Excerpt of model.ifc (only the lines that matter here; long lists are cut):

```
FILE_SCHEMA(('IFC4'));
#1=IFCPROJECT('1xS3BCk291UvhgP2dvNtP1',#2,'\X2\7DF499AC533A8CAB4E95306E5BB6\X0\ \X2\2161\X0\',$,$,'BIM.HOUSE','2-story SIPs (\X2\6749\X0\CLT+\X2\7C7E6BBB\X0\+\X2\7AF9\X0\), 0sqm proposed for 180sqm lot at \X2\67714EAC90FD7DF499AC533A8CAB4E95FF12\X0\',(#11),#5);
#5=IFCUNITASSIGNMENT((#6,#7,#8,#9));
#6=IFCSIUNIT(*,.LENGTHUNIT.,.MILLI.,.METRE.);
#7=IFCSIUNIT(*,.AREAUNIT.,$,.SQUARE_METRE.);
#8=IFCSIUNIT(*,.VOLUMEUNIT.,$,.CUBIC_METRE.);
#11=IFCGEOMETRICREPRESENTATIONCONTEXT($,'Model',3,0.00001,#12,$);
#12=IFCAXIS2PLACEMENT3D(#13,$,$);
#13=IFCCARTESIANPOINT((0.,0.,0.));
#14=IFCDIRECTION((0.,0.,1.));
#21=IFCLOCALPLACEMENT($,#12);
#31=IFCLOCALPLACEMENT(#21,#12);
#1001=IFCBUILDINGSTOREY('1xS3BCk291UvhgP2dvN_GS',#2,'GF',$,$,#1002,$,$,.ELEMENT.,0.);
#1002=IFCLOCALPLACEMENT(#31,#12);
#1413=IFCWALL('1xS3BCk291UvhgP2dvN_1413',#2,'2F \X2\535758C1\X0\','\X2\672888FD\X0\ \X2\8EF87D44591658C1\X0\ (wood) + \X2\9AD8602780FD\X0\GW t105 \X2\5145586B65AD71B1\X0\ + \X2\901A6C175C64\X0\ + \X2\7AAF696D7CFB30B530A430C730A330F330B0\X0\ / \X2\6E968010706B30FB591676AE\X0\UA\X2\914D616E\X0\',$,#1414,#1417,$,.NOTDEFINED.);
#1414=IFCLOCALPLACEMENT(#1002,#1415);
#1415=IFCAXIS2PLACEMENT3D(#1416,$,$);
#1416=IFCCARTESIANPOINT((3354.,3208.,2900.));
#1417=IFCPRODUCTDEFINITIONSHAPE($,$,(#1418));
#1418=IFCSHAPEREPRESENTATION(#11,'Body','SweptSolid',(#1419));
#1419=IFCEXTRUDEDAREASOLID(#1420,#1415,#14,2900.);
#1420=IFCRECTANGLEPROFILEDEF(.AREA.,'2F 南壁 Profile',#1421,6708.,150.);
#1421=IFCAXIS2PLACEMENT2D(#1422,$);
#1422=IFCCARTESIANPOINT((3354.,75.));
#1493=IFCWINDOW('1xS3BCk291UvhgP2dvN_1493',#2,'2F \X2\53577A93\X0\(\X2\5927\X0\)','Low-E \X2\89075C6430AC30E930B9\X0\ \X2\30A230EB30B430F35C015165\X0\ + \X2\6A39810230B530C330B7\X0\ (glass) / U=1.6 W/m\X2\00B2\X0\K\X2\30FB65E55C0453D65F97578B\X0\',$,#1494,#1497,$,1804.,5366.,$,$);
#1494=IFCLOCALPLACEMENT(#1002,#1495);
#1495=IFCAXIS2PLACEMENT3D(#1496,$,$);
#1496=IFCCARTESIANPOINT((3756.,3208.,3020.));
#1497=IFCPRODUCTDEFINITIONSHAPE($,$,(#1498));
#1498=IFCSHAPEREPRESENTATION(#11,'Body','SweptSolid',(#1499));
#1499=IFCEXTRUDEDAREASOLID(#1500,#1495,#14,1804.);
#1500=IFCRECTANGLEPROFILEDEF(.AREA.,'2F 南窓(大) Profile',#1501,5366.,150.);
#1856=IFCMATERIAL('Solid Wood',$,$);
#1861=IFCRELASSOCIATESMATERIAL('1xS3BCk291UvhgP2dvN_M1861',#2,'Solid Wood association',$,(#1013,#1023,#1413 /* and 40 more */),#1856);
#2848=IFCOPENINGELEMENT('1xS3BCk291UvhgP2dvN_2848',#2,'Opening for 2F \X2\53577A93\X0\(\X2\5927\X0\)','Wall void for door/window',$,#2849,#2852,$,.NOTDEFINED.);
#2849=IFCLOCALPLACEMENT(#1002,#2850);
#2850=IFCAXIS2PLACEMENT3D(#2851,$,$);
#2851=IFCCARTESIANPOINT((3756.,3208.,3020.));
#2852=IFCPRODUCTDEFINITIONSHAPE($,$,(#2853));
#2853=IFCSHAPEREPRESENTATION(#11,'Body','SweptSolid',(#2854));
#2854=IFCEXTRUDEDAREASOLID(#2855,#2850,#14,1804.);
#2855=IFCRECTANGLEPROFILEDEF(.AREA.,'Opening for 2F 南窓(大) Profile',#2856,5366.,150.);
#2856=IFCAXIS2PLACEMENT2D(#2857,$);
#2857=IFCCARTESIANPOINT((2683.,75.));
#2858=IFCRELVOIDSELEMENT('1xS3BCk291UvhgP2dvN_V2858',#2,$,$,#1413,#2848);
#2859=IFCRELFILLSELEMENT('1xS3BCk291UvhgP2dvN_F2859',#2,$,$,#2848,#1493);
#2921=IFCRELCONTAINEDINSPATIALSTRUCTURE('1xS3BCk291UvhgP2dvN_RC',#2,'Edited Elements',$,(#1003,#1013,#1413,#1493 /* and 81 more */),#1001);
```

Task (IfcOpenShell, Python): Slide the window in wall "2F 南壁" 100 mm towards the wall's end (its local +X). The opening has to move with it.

```python
import ifcopenshell
import ifcopenshell.api.geometry
import ifcopenshell.util.placement
import ifcopenshell.util.unit

model = ifcopenshell.open("model.ifc")
unit_scale = ifcopenshell.util.unit.calculate_unit_scale(model)

window = model.by_guid("1xS3BCk291UvhgP2dvN_1493")
opening = window.FillsVoids[0].RelatingOpeningElement
wall = opening.VoidsElements[0].RelatingBuildingElement

wall_matrix = ifcopenshell.util.placement.get_local_placement(wall.ObjectPlacement)
shift = wall_matrix[:3, 0] * 0.1 / unit_scale
before = ifcopenshell.util.placement.get_local_placement(window.ObjectPlacement)[:3, 3].copy()

# The window is not placed relative to its opening, so move both.
for product in (opening, window):
    matrix = ifcopenshell.util.placement.get_local_placement(product.ObjectPlacement)
    matrix[:3, 3] += shift
    ifcopenshell.api.geometry.edit_object_placement(model, product=product, matrix=matrix, is_si=False)

after = ifcopenshell.util.placement.get_local_placement(window.ObjectPlacement)[:3, 3]
print("window moved by", (after - before).round(3) + 0.0)

model.write("model_edited.ifc")
```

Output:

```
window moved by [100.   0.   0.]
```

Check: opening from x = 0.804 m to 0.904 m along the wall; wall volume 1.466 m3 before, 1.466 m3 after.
